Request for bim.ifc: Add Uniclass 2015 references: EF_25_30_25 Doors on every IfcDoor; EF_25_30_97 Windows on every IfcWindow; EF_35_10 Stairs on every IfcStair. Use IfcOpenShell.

First a look at what the model holds.

```python
import ifcopenshell

model = ifcopenshell.open("bim.ifc")
print(model.schema)
print("classifications:", [c.Name for c in model.by_type("IfcClassification")])
for ifc_class in ("IfcDoor", "IfcRoof", "IfcStair", "IfcWall", "IfcWindow"):
    print(ifc_class, len(model.by_type(ifc_class)))
```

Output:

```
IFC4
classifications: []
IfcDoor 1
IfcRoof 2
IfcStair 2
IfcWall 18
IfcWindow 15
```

```python
import ifcopenshell
import ifcopenshell.api.classification

model = ifcopenshell.open("bim.ifc")

system = ifcopenshell.api.classification.add_classification(model, classification="Uniclass 2015")

codes = {
    "IfcDoor": ("EF_25_30_25", "Doors"),
    "IfcWindow": ("EF_25_30_97", "Windows"),
    "IfcStair": ("EF_35_10", "Stairs"),
}
for ifc_class, (code, name) in codes.items():
    products = model.by_type(ifc_class)
    ifcopenshell.api.classification.add_reference(
        model, products=products, classification=system, identification=code, name=name
    )
    print(code, len(products))

model.write("bim_edited.ifc")
```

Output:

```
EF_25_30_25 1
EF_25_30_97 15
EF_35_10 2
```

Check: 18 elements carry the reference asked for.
